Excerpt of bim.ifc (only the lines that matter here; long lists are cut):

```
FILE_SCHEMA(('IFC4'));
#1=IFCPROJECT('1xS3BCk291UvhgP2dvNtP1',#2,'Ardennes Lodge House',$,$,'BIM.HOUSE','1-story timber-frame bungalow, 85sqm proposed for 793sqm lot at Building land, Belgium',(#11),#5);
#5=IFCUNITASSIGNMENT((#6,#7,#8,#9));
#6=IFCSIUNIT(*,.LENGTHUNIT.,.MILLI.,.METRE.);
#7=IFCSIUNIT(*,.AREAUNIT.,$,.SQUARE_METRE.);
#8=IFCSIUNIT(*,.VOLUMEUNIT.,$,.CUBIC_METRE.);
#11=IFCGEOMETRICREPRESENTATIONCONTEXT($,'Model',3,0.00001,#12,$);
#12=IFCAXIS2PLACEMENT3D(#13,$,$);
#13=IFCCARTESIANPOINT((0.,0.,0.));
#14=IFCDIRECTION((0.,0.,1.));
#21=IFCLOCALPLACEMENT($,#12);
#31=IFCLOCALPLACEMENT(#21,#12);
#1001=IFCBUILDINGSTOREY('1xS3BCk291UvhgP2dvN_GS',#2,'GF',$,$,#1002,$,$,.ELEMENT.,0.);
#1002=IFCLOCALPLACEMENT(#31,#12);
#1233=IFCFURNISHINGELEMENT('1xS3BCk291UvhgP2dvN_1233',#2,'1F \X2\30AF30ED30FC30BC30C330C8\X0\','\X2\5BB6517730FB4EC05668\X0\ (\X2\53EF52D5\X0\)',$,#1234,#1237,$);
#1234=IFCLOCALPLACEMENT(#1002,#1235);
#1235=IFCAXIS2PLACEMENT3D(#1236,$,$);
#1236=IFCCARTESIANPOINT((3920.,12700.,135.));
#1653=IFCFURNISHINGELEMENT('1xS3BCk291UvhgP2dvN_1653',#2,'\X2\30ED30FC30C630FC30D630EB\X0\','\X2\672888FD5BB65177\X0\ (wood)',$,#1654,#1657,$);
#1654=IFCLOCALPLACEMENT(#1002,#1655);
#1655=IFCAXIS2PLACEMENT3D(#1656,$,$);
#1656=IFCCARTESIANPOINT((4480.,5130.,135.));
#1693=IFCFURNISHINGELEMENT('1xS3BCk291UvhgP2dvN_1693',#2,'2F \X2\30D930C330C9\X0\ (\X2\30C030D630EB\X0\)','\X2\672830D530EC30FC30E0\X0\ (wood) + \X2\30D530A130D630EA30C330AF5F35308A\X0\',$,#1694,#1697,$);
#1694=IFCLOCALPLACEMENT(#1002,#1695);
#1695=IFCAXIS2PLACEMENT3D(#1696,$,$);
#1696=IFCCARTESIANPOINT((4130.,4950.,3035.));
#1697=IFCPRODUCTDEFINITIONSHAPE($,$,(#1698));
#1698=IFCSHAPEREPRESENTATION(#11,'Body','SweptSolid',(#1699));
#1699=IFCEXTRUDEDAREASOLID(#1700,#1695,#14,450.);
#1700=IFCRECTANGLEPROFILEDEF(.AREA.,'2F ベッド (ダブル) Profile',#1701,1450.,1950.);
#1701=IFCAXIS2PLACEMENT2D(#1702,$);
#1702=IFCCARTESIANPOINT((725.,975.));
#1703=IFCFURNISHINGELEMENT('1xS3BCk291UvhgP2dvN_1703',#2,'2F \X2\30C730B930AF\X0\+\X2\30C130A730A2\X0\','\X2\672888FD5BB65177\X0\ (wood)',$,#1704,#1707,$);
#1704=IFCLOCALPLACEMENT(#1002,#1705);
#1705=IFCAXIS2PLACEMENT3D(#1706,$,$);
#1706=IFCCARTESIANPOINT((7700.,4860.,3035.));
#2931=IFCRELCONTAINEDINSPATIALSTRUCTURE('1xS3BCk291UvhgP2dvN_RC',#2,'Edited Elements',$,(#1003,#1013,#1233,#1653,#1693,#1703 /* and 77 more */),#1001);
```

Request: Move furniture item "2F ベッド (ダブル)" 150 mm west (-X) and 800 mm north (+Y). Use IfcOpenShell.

```python
import ifcopenshell
import ifcopenshell.api.geometry
import ifcopenshell.util.placement
import ifcopenshell.util.unit

model = ifcopenshell.open("bim.ifc")
unit_scale = ifcopenshell.util.unit.calculate_unit_scale(model)

item = model.by_guid("1xS3BCk291UvhgP2dvN_1693")
matrix = ifcopenshell.util.placement.get_local_placement(item.ObjectPlacement)
matrix[0, 3] -= 0.15 / unit_scale
matrix[1, 3] += 0.8 / unit_scale
ifcopenshell.api.geometry.edit_object_placement(model, product=item, matrix=matrix, is_si=False)

print(ifcopenshell.util.placement.get_local_placement(item.ObjectPlacement).round(3) + 0.0)

model.write("bim_edited.ifc")
```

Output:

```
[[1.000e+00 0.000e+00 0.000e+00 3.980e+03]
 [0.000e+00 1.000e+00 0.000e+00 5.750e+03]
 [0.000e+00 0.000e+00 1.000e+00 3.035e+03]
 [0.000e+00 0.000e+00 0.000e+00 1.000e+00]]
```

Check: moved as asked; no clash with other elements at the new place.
